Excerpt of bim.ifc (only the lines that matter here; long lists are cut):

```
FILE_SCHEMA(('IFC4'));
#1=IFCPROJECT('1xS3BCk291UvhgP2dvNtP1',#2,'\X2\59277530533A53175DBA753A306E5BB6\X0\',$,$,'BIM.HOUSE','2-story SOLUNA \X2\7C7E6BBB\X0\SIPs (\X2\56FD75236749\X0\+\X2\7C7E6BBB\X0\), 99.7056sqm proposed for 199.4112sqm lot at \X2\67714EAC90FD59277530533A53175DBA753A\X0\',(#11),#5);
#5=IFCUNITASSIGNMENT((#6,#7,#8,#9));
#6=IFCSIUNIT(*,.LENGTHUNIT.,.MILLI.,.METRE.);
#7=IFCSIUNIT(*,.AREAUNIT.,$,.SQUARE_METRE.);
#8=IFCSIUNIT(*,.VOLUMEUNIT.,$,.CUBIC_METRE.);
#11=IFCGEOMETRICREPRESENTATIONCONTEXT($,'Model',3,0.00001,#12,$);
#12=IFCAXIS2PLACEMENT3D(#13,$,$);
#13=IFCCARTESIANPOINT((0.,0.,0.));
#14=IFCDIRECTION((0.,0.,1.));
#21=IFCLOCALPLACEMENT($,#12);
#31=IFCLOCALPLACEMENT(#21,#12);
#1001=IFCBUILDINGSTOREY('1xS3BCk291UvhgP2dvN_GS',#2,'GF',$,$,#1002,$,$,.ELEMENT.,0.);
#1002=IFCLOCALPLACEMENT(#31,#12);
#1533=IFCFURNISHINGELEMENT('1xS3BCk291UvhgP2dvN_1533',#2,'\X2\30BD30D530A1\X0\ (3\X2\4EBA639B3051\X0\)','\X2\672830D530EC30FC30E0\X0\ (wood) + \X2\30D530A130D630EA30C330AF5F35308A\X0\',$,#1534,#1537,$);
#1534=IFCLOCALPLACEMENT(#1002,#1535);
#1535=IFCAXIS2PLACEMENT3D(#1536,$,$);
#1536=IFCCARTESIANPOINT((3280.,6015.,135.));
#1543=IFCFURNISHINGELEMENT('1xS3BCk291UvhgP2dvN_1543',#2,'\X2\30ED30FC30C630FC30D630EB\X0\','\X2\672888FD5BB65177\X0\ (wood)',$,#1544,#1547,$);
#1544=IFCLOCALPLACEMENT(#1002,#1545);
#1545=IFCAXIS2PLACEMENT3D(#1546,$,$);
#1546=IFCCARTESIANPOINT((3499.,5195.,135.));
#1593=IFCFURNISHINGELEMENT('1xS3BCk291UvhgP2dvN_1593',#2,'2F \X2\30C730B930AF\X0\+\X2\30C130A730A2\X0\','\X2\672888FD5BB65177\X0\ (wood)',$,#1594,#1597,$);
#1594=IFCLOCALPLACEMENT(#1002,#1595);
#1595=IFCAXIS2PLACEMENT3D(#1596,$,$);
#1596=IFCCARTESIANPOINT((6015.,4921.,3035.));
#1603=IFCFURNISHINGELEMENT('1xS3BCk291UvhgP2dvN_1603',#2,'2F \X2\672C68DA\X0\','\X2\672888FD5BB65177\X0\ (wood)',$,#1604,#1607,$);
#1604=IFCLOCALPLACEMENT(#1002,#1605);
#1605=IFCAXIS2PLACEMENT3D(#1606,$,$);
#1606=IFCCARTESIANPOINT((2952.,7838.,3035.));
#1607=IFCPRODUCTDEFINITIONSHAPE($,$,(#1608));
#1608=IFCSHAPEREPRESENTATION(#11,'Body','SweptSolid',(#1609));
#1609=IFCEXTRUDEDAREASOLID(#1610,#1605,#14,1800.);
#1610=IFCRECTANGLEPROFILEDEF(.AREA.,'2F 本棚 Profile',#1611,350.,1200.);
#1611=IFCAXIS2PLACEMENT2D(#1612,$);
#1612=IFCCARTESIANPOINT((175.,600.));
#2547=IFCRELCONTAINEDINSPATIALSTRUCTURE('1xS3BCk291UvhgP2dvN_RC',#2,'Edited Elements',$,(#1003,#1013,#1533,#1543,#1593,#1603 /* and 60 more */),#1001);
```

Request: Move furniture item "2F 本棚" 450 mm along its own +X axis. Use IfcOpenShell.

```python
import ifcopenshell
import ifcopenshell.api.geometry
import ifcopenshell.util.placement

model = ifcopenshell.open("bim.ifc")

item = model.by_guid("1xS3BCk291UvhgP2dvN_1603")
matrix = ifcopenshell.util.placement.get_local_placement(item.ObjectPlacement)
matrix[:3, 3] += matrix[:3, 0] * 450.0
ifcopenshell.api.geometry.edit_object_placement(model, product=item, matrix=matrix, is_si=False)

print(ifcopenshell.util.placement.get_local_placement(item.ObjectPlacement).round(3) + 0.0)

model.write("bim_v2.ifc")
```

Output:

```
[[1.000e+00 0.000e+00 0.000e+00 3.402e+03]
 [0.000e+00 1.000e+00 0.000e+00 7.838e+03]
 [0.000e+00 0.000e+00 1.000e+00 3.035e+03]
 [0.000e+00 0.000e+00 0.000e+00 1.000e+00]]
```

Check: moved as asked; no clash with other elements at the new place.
